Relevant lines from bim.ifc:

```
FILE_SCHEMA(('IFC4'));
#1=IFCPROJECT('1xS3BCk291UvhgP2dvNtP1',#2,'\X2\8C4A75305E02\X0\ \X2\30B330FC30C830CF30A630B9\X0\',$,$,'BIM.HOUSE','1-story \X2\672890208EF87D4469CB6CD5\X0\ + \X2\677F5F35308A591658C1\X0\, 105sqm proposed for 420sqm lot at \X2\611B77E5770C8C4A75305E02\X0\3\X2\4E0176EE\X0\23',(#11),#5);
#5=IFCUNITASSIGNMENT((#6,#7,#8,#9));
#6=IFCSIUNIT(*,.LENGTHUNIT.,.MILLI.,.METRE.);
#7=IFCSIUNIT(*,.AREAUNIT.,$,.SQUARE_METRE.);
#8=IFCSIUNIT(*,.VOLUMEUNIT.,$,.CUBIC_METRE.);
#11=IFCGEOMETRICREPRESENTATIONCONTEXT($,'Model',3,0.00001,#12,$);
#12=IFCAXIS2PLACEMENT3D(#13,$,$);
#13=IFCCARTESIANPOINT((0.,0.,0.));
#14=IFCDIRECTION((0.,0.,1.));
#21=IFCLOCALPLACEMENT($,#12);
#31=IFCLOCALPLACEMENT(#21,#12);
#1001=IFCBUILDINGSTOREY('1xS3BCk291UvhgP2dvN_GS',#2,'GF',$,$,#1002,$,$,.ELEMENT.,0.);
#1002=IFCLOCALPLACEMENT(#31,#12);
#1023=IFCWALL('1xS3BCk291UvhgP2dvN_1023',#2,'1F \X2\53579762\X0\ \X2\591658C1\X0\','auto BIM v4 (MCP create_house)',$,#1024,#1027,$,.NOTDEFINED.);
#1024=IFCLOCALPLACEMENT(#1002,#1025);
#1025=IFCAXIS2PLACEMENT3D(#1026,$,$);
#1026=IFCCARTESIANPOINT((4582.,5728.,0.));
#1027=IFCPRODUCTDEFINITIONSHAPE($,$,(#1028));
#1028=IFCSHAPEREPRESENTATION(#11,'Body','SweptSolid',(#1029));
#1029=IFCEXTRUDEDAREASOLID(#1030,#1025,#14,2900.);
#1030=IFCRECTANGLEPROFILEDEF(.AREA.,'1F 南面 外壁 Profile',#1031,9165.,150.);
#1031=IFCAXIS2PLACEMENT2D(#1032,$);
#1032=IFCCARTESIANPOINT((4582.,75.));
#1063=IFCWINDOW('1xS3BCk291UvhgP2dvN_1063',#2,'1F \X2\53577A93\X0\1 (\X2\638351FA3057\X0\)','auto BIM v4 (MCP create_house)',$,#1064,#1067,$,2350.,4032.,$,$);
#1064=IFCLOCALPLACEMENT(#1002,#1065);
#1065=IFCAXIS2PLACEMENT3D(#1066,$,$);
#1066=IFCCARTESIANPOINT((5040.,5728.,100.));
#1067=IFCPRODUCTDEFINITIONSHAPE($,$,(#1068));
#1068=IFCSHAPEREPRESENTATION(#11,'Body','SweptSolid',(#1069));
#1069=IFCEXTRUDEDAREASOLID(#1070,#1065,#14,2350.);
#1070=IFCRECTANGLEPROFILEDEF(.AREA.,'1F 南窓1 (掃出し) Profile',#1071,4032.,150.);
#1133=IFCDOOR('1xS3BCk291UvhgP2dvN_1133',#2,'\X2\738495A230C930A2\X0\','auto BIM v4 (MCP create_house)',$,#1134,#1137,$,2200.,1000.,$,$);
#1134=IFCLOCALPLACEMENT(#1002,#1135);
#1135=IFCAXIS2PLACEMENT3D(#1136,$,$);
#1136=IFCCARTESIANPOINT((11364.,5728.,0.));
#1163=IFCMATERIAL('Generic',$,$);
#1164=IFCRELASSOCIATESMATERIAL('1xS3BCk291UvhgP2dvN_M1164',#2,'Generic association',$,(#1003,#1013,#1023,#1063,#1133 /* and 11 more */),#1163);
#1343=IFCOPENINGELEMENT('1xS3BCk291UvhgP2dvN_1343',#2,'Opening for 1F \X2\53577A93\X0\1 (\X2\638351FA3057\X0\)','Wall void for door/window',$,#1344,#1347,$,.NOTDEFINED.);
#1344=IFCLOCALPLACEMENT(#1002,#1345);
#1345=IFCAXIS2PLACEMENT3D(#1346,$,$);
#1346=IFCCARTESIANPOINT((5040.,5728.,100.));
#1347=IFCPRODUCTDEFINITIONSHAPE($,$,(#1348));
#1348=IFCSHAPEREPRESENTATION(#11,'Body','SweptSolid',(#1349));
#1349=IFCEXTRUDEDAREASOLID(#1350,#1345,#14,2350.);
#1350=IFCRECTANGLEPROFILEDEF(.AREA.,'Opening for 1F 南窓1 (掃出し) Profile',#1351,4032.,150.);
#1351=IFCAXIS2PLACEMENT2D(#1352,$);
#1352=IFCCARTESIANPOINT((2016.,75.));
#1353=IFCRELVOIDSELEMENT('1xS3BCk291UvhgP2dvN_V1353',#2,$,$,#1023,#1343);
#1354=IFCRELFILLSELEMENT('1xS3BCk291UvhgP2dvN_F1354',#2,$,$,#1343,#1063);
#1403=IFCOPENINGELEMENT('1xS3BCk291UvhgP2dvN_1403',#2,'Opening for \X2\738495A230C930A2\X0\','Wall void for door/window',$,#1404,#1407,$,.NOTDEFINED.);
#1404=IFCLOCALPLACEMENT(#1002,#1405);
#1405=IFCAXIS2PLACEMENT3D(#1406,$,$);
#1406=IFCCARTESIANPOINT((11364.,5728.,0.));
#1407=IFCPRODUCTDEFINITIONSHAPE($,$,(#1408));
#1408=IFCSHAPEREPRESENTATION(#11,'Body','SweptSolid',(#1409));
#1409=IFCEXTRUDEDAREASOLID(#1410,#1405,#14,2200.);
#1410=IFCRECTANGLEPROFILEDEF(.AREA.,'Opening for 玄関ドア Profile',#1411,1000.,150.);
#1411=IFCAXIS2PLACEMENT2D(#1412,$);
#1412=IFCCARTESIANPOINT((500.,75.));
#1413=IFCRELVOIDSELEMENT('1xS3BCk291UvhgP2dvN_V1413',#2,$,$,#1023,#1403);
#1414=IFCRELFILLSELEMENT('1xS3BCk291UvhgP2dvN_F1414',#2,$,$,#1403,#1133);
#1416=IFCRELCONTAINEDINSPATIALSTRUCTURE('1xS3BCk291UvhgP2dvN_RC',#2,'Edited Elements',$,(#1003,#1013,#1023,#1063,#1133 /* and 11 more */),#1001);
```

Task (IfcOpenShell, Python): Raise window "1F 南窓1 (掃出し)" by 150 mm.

```python
import numpy as np
import ifcopenshell
import ifcopenshell.api.geometry
import ifcopenshell.util.placement
import ifcopenshell.util.unit

model = ifcopenshell.open("bim.ifc")
unit_scale = ifcopenshell.util.unit.calculate_unit_scale(model)

window = model.by_id(1063)
opening = window.FillsVoids[0].RelatingOpeningElement
dz = 0.15 / unit_scale

shift = np.array([0.0, 0.0, dz])
# The window is not placed relative to its opening, so move both.
for product in (opening, window):
    matrix = ifcopenshell.util.placement.get_local_placement(product.ObjectPlacement)
    matrix[:3, 3] += shift
    ifcopenshell.api.geometry.edit_object_placement(model, product=product, matrix=matrix, is_si=False)

print(f"moved by {dz * unit_scale:+.3f} m")

model.write("bim_edited.ifc")
```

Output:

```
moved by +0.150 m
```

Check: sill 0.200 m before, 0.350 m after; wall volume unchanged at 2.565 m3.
